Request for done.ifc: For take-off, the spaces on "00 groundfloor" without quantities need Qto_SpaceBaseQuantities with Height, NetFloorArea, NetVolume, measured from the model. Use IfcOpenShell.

First a look at what the model holds.

```python
import ifcopenshell
import ifcopenshell.util.element
import ifcopenshell.util.unit

model = ifcopenshell.open("done.ifc")
print(model.schema)
for unit_type in ("LENGTHUNIT", "AREAUNIT", "VOLUMEUNIT"):
    print(unit_type, ifcopenshell.util.unit.calculate_unit_scale(model, unit_type))
storey = next(s for s in model.by_type("IfcBuildingStorey") if s.Name == "00 groundfloor")
spaces = [e for e in ifcopenshell.util.element.get_decomposition(storey) if e.is_a("IfcSpace")]
for e in sorted(spaces, key=lambda e: e.id()):
    print(e.id(), e.is_a(), e.Name, list(ifcopenshell.util.element.get_psets(e, qtos_only=True)), sep=" | ")
```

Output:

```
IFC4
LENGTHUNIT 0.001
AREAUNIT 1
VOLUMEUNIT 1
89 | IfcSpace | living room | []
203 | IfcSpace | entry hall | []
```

```python
import ifcopenshell
import ifcopenshell.api.pset
import ifcopenshell.geom
import ifcopenshell.util.element
import ifcopenshell.util.shape
import ifcopenshell.util.unit

model = ifcopenshell.open("done.ifc")
unit_scale = ifcopenshell.util.unit.calculate_unit_scale(model)
area_scale = ifcopenshell.util.unit.calculate_unit_scale(model, "AREAUNIT")
volume_scale = ifcopenshell.util.unit.calculate_unit_scale(model, "VOLUMEUNIT")
settings = ifcopenshell.geom.settings()

storey = next(s for s in model.by_type("IfcBuildingStorey") if s.Name == "00 groundfloor")
spaces = [e for e in ifcopenshell.util.element.get_decomposition(storey) if e.is_a("IfcSpace")]

for e in sorted(spaces, key=lambda e: e.id()):
    if ifcopenshell.util.element.get_psets(e, qtos_only=True, should_inherit=False):
        continue
    # Geometry comes back in metres, in the element's own axes.
    shape = ifcopenshell.geom.create_shape(settings, e)
    values = {
        "Height": ifcopenshell.util.shape.get_z(shape.geometry) / unit_scale,
        "NetFloorArea": ifcopenshell.util.shape.get_footprint_area(shape.geometry) / area_scale,
        "NetVolume": ifcopenshell.util.shape.get_volume(shape.geometry) / volume_scale,
    }
    qto = ifcopenshell.api.pset.add_qto(model, product=e, name="Qto_SpaceBaseQuantities")
    ifcopenshell.api.pset.edit_qto(model, qto=qto, properties=values)
    print(e.id(), {k: round(v, 3) for k, v in values.items()})

model.write("done_updated.ifc")
```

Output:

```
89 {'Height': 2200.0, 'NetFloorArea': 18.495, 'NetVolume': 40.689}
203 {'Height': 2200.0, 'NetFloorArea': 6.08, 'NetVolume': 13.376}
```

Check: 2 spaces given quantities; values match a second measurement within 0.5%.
